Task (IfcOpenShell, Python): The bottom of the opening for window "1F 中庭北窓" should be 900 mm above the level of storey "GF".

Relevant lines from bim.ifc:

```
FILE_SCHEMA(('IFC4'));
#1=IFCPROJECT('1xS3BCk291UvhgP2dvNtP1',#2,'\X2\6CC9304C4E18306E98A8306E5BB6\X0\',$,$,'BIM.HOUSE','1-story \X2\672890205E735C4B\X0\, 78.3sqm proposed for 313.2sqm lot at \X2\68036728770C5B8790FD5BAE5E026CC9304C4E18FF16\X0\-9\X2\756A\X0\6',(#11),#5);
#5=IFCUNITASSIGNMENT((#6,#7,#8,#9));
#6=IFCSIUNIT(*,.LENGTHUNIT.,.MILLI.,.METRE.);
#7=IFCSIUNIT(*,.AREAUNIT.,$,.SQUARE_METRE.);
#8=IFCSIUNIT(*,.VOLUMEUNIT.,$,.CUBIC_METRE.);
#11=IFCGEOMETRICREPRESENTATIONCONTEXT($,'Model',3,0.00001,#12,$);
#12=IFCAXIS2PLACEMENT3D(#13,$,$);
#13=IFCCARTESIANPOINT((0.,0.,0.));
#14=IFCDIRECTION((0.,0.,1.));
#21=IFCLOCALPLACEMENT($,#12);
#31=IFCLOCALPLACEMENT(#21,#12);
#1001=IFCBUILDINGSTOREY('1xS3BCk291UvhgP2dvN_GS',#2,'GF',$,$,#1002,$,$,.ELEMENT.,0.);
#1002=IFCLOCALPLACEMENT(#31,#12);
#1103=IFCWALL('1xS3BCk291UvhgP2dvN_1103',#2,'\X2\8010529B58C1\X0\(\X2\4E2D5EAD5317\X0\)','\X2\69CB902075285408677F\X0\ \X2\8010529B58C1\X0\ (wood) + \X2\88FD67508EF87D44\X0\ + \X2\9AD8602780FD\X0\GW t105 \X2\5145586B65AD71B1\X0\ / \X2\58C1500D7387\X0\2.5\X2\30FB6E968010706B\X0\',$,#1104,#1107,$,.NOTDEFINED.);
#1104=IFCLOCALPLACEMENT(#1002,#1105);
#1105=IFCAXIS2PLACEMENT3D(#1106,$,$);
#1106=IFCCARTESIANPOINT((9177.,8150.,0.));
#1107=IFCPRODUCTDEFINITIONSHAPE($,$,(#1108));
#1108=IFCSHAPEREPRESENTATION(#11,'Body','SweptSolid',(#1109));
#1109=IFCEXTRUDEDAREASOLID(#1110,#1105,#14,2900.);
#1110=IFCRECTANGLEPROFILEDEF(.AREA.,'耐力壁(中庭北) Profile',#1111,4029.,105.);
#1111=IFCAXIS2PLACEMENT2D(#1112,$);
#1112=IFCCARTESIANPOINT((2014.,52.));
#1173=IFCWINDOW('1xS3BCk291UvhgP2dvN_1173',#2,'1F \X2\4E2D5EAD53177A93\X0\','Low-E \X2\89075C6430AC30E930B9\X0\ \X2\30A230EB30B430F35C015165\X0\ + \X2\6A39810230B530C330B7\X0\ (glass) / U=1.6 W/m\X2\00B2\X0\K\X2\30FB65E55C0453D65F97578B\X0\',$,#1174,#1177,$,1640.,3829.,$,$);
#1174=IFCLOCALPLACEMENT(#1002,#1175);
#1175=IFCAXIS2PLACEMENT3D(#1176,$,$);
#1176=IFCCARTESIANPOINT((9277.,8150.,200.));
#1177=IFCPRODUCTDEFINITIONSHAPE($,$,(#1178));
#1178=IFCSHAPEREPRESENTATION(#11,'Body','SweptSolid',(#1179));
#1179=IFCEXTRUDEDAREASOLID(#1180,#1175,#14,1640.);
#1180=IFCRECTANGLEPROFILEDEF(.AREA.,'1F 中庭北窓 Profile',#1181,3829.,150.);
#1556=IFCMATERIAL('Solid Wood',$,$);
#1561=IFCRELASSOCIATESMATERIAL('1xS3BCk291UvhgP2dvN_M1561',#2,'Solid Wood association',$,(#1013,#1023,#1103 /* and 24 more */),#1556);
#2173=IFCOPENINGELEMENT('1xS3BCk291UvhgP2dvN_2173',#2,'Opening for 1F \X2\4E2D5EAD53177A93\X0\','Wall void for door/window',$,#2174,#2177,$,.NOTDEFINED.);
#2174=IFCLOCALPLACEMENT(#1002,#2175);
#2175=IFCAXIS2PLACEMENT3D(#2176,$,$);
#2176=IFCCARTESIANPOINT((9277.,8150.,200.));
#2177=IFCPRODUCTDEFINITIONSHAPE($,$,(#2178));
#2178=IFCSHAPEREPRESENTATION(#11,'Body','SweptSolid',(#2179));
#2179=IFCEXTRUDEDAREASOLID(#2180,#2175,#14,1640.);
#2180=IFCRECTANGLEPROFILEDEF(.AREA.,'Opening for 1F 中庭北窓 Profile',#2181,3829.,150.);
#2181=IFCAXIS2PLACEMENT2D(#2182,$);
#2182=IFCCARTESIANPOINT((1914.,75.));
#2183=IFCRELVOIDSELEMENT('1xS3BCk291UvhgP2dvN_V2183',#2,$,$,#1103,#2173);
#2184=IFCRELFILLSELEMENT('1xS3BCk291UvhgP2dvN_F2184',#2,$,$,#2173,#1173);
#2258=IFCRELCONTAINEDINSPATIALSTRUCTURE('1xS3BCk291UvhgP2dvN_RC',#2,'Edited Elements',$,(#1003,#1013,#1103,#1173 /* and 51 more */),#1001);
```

```python
import numpy as np
import ifcopenshell
import ifcopenshell.api.geometry
import ifcopenshell.geom
import ifcopenshell.util.element
import ifcopenshell.util.placement
import ifcopenshell.util.shape
import ifcopenshell.util.unit

model = ifcopenshell.open("bim.ifc")
unit_scale = ifcopenshell.util.unit.calculate_unit_scale(model)

window = model.by_id(1173)
opening = window.FillsVoids[0].RelatingOpeningElement
storey = ifcopenshell.util.element.get_container(window, ifc_class="IfcBuildingStorey")
level = ifcopenshell.util.placement.get_local_placement(storey.ObjectPlacement)[2, 3]

# The opening's origin need not be at the sill, so measure its lowest point.
shape = ifcopenshell.geom.create_shape(ifcopenshell.geom.settings(), opening)
bottom = ifcopenshell.util.shape.get_shape_bottom_elevation(shape, shape.geometry) / unit_scale
dz = level + 0.9 / unit_scale - bottom

shift = np.array([0.0, 0.0, dz])
# The window is not placed relative to its opening, so move both.
for product in (opening, window):
    matrix = ifcopenshell.util.placement.get_local_placement(product.ObjectPlacement)
    matrix[:3, 3] += shift
    ifcopenshell.api.geometry.edit_object_placement(model, product=product, matrix=matrix, is_si=False)

print(f"moved by {dz * unit_scale:+.3f} m")

model.write("bim_edited.ifc")
```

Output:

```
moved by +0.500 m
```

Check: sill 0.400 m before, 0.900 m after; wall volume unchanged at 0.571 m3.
